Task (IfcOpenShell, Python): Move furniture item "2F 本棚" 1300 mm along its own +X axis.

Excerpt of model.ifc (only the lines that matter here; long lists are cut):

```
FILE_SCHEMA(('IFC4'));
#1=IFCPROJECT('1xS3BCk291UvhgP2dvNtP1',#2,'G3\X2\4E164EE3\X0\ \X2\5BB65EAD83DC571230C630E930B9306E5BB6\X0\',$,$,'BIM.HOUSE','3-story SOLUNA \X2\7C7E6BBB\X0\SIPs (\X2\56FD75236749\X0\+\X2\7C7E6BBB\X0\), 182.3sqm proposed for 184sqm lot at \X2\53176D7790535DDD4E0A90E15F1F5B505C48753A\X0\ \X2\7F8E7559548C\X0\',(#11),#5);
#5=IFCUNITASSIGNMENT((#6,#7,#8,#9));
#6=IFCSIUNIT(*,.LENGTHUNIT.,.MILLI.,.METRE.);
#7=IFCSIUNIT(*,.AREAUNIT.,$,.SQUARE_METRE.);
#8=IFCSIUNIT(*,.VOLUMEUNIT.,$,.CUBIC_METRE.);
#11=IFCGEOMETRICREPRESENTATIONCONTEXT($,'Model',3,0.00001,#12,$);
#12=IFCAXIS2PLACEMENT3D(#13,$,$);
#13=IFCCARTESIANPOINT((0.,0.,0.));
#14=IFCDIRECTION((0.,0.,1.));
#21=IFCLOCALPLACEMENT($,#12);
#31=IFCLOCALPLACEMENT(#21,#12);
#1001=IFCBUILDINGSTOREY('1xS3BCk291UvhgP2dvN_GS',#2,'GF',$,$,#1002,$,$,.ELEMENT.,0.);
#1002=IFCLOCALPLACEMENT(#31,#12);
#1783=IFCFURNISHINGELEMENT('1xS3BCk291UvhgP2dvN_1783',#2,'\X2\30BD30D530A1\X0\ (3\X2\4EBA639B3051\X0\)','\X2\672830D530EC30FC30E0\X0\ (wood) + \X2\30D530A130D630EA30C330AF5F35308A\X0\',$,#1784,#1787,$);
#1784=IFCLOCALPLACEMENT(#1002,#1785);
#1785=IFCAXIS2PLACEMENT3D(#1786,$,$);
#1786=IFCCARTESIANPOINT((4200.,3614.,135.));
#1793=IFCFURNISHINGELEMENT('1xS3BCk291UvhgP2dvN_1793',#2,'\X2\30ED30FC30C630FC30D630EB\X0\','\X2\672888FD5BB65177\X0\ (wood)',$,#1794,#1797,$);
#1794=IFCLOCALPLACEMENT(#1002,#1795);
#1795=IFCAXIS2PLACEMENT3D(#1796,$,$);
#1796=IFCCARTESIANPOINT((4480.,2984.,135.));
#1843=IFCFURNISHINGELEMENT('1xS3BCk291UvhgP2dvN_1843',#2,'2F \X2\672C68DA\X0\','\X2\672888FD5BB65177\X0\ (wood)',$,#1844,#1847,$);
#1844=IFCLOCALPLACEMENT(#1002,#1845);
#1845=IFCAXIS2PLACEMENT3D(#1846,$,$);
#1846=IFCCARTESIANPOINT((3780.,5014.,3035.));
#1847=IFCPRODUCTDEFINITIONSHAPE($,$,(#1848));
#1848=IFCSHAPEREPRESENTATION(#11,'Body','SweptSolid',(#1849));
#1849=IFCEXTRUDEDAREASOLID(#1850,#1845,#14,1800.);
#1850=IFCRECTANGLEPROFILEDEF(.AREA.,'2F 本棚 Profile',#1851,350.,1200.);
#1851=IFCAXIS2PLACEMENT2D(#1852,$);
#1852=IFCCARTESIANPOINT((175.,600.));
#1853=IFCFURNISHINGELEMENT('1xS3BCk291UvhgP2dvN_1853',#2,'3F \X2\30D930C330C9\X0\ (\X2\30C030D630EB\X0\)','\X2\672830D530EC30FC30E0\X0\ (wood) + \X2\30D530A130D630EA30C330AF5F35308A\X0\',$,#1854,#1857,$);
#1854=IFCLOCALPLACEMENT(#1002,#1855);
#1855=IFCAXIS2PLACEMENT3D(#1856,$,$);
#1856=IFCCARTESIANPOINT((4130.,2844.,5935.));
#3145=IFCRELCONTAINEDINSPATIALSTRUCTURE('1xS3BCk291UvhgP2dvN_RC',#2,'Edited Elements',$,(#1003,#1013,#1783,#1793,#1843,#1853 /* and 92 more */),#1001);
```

```python
import ifcopenshell
import ifcopenshell.api.geometry
import ifcopenshell.util.placement

model = ifcopenshell.open("model.ifc")

item = model.by_guid("1xS3BCk291UvhgP2dvN_1843")
matrix = ifcopenshell.util.placement.get_local_placement(item.ObjectPlacement)
matrix[:3, 3] += matrix[:3, 0] * 1300.0
ifcopenshell.api.geometry.edit_object_placement(model, product=item, matrix=matrix, is_si=False)

print(ifcopenshell.util.placement.get_local_placement(item.ObjectPlacement).round(3) + 0.0)

model.write("model_edited.ifc")
```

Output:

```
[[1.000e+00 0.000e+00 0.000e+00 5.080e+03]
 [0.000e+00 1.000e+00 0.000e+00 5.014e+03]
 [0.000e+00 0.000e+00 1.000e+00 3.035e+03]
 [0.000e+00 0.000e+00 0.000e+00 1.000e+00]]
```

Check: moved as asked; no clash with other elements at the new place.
